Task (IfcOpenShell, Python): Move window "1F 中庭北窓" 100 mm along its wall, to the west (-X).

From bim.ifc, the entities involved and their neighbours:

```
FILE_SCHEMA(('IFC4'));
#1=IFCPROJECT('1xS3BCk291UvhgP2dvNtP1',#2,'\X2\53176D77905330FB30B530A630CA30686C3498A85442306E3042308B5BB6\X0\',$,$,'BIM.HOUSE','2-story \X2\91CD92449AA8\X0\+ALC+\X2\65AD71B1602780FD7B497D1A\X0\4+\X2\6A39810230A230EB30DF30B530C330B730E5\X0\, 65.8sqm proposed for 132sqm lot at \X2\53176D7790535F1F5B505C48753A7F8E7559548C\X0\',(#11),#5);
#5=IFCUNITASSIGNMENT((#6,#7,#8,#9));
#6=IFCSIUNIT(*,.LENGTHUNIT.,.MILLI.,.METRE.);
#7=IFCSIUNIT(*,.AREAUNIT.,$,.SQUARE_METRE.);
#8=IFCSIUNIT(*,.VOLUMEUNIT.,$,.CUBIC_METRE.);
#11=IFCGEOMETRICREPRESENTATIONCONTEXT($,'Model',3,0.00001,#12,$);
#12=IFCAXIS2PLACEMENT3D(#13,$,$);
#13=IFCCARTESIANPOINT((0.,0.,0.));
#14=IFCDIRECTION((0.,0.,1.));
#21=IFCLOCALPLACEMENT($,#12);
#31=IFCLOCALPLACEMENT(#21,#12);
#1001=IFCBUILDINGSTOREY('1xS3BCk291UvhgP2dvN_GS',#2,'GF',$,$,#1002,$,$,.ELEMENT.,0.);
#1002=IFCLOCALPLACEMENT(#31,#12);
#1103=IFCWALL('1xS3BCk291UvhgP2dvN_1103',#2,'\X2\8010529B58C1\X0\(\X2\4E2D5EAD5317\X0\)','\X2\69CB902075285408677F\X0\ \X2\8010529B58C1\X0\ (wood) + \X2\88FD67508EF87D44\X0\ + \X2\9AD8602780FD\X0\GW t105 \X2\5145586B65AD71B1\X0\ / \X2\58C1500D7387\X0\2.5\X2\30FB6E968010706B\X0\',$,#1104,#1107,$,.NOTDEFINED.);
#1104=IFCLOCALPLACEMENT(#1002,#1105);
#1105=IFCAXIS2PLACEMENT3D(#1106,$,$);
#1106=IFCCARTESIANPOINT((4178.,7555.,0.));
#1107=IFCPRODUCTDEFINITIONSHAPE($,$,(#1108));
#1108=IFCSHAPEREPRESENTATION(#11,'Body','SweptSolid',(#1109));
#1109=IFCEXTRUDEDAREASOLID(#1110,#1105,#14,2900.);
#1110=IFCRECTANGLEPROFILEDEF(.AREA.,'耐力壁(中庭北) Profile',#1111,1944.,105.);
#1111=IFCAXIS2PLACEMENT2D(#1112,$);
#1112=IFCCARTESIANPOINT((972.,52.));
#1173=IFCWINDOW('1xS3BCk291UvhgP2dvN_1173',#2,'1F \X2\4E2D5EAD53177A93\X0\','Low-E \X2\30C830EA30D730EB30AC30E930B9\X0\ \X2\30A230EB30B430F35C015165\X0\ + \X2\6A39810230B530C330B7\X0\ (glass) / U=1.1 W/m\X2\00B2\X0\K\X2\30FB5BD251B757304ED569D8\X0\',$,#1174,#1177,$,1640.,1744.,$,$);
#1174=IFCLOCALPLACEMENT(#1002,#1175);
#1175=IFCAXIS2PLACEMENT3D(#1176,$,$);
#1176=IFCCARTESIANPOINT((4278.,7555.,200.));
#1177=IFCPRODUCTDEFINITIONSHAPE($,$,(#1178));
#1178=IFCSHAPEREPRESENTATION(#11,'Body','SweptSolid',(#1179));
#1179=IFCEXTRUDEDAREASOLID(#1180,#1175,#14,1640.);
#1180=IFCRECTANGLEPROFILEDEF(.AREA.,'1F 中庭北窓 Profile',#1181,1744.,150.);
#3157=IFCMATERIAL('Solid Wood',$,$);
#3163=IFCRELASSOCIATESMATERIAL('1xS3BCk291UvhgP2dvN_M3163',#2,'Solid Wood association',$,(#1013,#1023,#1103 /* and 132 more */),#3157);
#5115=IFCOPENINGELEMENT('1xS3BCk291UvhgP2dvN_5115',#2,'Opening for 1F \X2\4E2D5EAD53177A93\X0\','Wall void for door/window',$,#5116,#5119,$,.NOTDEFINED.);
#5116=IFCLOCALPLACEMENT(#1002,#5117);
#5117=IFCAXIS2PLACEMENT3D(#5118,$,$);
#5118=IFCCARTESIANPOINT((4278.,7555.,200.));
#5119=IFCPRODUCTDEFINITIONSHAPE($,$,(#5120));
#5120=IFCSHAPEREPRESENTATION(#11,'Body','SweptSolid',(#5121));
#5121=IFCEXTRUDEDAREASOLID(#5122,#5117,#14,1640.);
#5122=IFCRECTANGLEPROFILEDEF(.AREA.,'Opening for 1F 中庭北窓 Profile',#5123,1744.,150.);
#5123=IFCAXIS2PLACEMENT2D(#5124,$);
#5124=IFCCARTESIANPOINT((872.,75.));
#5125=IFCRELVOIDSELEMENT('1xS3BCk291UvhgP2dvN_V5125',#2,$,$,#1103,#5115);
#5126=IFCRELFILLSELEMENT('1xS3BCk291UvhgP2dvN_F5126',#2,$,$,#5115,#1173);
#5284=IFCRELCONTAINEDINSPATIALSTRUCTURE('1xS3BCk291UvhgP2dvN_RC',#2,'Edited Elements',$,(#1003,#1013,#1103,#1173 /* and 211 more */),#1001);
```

```python
import ifcopenshell
import ifcopenshell.api.geometry
import ifcopenshell.util.placement
import ifcopenshell.util.unit

model = ifcopenshell.open("bim.ifc")
unit_scale = ifcopenshell.util.unit.calculate_unit_scale(model)

window = model.by_guid("1xS3BCk291UvhgP2dvN_1173")
opening = window.FillsVoids[0].RelatingOpeningElement
wall = opening.VoidsElements[0].RelatingBuildingElement

wall_matrix = ifcopenshell.util.placement.get_local_placement(wall.ObjectPlacement)
shift = wall_matrix[:3, 0] * -0.1 / unit_scale
before = ifcopenshell.util.placement.get_local_placement(window.ObjectPlacement)[:3, 3].copy()

# The window is not placed relative to its opening, so move both.
for product in (opening, window):
    matrix = ifcopenshell.util.placement.get_local_placement(product.ObjectPlacement)
    matrix[:3, 3] += shift
    ifcopenshell.api.geometry.edit_object_placement(model, product=product, matrix=matrix, is_si=False)

after = ifcopenshell.util.placement.get_local_placement(window.ObjectPlacement)[:3, 3]
print("window moved by", (after - before).round(3) + 0.0)

model.write("bim_v2.ifc")
```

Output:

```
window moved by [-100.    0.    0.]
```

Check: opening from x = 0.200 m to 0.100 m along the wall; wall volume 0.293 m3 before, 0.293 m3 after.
